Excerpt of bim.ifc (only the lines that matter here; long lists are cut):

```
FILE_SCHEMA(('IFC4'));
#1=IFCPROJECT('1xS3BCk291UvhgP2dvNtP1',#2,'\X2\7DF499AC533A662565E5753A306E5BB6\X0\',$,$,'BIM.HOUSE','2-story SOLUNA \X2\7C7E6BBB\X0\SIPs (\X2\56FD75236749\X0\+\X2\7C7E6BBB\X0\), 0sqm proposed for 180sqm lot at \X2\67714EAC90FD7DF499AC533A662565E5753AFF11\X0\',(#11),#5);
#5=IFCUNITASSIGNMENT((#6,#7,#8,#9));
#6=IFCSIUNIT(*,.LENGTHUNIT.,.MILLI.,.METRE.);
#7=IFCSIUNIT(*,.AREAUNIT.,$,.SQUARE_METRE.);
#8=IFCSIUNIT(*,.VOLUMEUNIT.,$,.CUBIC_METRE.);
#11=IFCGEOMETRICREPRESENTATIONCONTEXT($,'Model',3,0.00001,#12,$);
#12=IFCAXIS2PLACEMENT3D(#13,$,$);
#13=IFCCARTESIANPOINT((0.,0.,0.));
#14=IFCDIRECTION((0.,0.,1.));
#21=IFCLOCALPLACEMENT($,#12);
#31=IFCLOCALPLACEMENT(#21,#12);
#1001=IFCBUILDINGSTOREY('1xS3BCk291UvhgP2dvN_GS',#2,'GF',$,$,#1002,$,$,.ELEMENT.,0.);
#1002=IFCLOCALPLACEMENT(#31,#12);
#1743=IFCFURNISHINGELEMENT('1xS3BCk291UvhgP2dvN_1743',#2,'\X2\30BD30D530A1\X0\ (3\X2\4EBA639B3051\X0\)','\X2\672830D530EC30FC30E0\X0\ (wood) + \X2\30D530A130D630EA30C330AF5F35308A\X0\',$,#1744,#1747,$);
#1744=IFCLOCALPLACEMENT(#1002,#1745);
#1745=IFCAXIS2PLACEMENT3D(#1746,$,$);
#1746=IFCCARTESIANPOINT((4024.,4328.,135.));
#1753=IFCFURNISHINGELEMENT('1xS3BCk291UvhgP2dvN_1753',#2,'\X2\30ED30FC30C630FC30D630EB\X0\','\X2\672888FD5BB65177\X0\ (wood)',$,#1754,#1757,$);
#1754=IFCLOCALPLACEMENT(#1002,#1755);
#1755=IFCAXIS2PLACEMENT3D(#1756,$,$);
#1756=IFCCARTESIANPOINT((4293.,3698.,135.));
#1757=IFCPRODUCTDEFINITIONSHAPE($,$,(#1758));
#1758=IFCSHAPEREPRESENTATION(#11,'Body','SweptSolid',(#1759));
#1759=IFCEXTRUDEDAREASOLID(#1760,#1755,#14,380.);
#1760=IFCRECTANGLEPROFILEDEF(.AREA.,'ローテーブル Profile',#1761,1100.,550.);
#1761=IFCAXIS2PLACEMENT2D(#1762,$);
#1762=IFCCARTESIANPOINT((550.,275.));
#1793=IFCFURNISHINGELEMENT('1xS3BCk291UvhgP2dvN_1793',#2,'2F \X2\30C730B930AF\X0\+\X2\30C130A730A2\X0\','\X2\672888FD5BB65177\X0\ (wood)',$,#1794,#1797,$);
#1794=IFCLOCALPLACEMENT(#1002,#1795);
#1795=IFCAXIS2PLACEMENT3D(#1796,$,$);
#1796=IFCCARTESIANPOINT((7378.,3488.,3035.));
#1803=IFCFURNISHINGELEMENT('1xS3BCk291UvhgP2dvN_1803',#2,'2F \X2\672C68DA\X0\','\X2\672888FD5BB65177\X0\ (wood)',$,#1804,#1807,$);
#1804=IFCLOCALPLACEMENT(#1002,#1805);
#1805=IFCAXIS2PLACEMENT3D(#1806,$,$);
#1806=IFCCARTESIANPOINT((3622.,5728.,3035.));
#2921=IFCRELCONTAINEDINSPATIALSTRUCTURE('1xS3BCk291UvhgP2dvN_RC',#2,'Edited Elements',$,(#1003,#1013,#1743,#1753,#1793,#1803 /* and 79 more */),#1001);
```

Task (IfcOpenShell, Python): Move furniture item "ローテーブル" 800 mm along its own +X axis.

```python
import ifcopenshell
import ifcopenshell.api.geometry
import ifcopenshell.util.placement

model = ifcopenshell.open("bim.ifc")

item = model.by_guid("1xS3BCk291UvhgP2dvN_1753")
matrix = ifcopenshell.util.placement.get_local_placement(item.ObjectPlacement)
matrix[:3, 3] += matrix[:3, 0] * 800.0
ifcopenshell.api.geometry.edit_object_placement(model, product=item, matrix=matrix, is_si=False)

print(ifcopenshell.util.placement.get_local_placement(item.ObjectPlacement).round(3) + 0.0)

model.write("bim_rev.ifc")
```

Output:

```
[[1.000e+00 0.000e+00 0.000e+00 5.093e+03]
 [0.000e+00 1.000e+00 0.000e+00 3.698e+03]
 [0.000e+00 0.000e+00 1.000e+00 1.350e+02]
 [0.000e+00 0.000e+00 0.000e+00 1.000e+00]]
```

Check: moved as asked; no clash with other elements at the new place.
